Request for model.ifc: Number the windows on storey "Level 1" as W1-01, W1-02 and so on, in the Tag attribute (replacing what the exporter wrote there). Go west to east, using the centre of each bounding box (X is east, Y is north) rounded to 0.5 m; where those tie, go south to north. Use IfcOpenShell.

First a look at what the model holds.

```python
import ifcopenshell
import ifcopenshell.util.element
import ifcopenshell.util.placement

model = ifcopenshell.open("model.ifc")
print(model.schema)
storey = next(s for s in model.by_type("IfcBuildingStorey") if s.Name == "Level 1")
windows = [e for e in ifcopenshell.util.element.get_decomposition(storey) if e.is_a("IfcWindow")]
for e in sorted(windows, key=lambda e: e.id()):
    origin = ifcopenshell.util.placement.get_local_placement(e.ObjectPlacement)[:3, 3]
    print(e.id(), e.Tag, e.Name, origin.round(2) + 0.0, sep=" | ")
```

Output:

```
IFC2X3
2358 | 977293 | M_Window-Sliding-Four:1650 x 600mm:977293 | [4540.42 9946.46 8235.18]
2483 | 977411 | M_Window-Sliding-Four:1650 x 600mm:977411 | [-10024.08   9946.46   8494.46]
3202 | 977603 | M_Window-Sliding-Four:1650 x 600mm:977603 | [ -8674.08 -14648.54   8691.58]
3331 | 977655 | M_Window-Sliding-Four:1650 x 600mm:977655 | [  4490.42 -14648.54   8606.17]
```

```python
import ifcopenshell
import ifcopenshell.geom
import ifcopenshell.util.element
import ifcopenshell.util.shape

model = ifcopenshell.open("model.ifc")
settings = ifcopenshell.geom.settings()
settings.set("use-world-coords", True)


def centre(element):
    shape = ifcopenshell.geom.create_shape(settings, element)
    return ifcopenshell.util.shape.get_bbox_centroid(shape.geometry)


storey = next(s for s in model.by_type("IfcBuildingStorey") if s.Name == "Level 1")
windows = [e for e in ifcopenshell.util.element.get_decomposition(storey) if e.is_a("IfcWindow")]

# Insertion points can sit at a corner or the storey origin, so sort by the geometry (in metres).
centres = {e: centre(e) for e in windows}
windows.sort(key=lambda e: (round(centres[e][0] / 0.5), centres[e][1]))

for i, e in enumerate(windows, start=1):
    number = f"W1-{i:02d}"
    e.Tag = number
    print(e.id(), number)

model.write("model_v2.ifc")
```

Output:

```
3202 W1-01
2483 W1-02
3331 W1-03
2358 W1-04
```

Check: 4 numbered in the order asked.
